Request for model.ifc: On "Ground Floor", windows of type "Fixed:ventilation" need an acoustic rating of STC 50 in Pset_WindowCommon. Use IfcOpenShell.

First a look at what the model holds.

```python
import ifcopenshell
import ifcopenshell.util.element

model = ifcopenshell.open("model.ifc")
print(model.schema)
storey = next(s for s in model.by_type("IfcBuildingStorey") if s.Name == "Ground Floor")
windows = [e for e in ifcopenshell.util.element.get_decomposition(storey) if e.is_a("IfcWindow")]
seen = {}
for e in windows:
    element_type = ifcopenshell.util.element.get_type(e)
    key = (element_type.Name if element_type != e and element_type else None, ifcopenshell.util.element.get_pset(e, "Pset_WindowCommon", "AcousticRating"))
    seen[key] = seen.get(key, 0) + 1
for (name, value), count in sorted(seen.items(), key=str):
    print(count, "x", name, "|", value)
```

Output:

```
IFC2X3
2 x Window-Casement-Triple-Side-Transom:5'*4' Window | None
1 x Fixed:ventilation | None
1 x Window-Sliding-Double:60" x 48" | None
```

```python
import ifcopenshell
import ifcopenshell.api.pset
import ifcopenshell.util.element

model = ifcopenshell.open("model.ifc")

storey = next(s for s in model.by_type("IfcBuildingStorey") if s.Name == "Ground Floor")
windows = [e for e in ifcopenshell.util.element.get_decomposition(storey) if e.is_a("IfcWindow")]

count = 0
for e in windows:
    element_type = ifcopenshell.util.element.get_type(e)
    if element_type in (None, e) or element_type.Name != "Fixed:ventilation":
        continue
    # add_pset returns the element's existing set when there is one.
    pset = ifcopenshell.api.pset.add_pset(model, product=e, name="Pset_WindowCommon")
    ifcopenshell.api.pset.edit_pset(model, pset=pset, properties={"AcousticRating": "STC 50"})
    count += 1

print(count, "windows updated")

model.write("model_edited.ifc")
```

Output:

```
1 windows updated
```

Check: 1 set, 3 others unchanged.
